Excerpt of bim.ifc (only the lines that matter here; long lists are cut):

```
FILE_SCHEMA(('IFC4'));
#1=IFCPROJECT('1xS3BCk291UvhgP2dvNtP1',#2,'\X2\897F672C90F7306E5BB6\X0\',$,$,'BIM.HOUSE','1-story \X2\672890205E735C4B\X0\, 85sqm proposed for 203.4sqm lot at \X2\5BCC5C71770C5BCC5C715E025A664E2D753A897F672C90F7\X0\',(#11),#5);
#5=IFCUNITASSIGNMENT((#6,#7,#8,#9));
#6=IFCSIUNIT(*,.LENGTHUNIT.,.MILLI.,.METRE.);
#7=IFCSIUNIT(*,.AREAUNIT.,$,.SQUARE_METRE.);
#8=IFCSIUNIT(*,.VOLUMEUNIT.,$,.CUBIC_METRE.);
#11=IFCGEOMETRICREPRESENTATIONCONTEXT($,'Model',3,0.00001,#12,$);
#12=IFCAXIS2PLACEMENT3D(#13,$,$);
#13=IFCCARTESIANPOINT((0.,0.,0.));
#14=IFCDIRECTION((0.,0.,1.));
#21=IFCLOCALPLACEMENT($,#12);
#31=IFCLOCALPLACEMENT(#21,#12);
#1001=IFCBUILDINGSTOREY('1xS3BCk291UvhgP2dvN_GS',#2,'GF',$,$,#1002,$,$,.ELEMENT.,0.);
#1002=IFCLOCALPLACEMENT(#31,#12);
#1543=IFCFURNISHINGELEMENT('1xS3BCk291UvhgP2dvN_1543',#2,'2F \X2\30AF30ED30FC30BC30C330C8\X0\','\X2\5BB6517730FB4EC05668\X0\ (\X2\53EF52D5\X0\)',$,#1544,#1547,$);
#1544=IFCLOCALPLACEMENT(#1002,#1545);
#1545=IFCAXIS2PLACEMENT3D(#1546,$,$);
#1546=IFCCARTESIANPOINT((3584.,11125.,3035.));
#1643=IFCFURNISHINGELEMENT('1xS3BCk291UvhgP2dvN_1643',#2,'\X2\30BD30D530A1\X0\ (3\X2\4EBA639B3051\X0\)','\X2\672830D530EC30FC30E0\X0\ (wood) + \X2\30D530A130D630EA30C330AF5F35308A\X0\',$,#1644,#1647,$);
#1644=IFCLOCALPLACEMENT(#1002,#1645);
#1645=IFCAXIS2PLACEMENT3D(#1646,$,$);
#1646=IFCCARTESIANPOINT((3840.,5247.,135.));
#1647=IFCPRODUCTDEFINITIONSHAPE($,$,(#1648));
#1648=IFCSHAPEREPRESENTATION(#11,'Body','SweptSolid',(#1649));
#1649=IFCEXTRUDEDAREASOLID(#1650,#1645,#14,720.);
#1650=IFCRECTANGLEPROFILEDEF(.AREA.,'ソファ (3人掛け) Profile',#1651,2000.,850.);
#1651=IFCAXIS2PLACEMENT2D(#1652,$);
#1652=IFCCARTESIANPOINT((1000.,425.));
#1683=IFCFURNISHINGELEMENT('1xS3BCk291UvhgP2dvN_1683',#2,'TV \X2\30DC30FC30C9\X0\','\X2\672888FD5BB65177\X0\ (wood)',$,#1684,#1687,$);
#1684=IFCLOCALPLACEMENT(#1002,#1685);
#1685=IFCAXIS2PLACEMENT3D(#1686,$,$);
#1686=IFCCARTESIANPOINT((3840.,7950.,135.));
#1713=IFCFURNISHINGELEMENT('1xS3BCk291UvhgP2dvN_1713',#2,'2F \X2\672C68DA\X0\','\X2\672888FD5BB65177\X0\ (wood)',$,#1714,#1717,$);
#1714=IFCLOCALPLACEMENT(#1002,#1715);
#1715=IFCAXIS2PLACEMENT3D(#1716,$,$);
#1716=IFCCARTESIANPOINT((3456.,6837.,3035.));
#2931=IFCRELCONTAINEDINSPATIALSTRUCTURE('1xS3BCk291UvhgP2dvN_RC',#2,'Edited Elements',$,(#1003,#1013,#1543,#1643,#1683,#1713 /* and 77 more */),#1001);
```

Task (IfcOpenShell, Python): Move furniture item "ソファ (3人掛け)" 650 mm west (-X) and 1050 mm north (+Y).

```python
import ifcopenshell
import ifcopenshell.api.geometry
import ifcopenshell.util.placement

model = ifcopenshell.open("bim.ifc")

item = model.by_id(1643)
matrix = ifcopenshell.util.placement.get_local_placement(item.ObjectPlacement)
matrix[0, 3] -= 650.0
matrix[1, 3] += 1050.0
ifcopenshell.api.geometry.edit_object_placement(model, product=item, matrix=matrix, is_si=False)

print(ifcopenshell.util.placement.get_local_placement(item.ObjectPlacement).round(3) + 0.0)

model.write("bim_rev.ifc")
```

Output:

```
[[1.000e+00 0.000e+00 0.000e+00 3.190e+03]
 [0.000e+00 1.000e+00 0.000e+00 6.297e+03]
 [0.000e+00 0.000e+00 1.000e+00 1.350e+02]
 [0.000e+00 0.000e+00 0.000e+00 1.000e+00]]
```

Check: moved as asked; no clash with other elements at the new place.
